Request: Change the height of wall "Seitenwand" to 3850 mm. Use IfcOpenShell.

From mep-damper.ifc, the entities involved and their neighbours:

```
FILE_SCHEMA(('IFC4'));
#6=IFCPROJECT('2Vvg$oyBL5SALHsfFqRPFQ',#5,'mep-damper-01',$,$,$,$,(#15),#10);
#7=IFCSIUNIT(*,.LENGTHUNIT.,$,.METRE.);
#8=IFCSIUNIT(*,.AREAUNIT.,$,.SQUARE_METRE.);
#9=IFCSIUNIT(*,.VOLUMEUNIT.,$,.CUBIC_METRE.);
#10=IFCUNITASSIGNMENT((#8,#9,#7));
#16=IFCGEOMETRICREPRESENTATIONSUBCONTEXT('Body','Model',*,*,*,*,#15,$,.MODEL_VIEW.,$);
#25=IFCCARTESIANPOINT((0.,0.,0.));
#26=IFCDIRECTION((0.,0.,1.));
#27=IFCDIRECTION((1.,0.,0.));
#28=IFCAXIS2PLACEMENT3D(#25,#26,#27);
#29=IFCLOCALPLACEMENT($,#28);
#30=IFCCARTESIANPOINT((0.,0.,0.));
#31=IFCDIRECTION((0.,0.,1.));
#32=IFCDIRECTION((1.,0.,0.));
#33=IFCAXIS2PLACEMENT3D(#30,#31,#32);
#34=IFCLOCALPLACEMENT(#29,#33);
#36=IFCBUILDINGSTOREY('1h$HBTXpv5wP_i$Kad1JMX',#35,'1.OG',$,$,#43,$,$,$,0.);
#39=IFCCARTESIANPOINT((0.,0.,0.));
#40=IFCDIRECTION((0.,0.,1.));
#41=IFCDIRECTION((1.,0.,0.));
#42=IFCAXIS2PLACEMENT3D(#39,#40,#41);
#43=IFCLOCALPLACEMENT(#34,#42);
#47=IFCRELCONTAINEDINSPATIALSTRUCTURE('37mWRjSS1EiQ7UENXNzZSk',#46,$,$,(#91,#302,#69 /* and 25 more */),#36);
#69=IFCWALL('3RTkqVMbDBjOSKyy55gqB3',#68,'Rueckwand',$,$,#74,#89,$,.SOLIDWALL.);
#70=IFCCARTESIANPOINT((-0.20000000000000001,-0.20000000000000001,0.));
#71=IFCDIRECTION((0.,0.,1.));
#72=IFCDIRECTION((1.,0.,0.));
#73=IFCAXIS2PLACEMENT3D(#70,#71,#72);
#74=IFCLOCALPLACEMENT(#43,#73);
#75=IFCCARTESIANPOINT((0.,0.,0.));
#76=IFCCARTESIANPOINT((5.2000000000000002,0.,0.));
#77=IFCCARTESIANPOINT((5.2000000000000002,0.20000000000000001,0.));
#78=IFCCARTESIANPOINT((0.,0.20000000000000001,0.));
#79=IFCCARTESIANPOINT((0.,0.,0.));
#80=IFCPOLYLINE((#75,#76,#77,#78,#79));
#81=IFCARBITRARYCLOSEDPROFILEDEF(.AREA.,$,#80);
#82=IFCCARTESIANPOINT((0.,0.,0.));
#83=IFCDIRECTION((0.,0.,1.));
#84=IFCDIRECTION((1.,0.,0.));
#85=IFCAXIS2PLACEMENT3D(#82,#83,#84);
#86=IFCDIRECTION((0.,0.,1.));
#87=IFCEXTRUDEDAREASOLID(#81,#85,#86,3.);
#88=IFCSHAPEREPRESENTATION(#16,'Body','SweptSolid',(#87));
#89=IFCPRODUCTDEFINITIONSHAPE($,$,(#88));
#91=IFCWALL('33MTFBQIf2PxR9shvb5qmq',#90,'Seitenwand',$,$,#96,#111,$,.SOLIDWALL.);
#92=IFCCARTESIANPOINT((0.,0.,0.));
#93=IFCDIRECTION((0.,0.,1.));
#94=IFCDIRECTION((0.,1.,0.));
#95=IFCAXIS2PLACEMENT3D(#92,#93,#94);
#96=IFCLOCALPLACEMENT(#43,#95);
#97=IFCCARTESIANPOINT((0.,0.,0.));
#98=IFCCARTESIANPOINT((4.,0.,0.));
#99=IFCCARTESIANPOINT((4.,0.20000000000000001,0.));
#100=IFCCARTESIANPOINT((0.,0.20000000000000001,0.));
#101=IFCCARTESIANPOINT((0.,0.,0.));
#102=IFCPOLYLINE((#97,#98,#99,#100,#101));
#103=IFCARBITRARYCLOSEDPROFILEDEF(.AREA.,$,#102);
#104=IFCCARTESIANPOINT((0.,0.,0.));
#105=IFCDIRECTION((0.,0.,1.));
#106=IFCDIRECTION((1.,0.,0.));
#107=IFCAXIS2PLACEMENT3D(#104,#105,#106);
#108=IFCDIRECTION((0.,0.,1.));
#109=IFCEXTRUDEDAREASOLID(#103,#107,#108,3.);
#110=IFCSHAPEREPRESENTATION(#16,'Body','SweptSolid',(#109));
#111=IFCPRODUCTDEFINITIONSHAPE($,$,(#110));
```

```python
import ifcopenshell
import ifcopenshell.geom
import ifcopenshell.util.representation
import ifcopenshell.util.shape

model = ifcopenshell.open("mep-damper.ifc")
settings = ifcopenshell.geom.settings()


def volume(element):
    """Net volume in cubic metres, openings subtracted."""
    shape = ifcopenshell.geom.create_shape(settings, element)
    return ifcopenshell.util.shape.get_volume(shape.geometry)


wall = model.by_guid("33MTFBQIf2PxR9shvb5qmq")
before = volume(wall)

body = ifcopenshell.util.representation.get_representation(wall, "Model", "Body")
solid = body.Items[0]
old_height = solid.Depth
solid.Depth = 3.85
after = volume(wall)

print(f"height {old_height:g} -> {solid.Depth:g}, volume {before:.3f} -> {after:.3f} m3")

model.write("mep-damper_rev.ifc")
```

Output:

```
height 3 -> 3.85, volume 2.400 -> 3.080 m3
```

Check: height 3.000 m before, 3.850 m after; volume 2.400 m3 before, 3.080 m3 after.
